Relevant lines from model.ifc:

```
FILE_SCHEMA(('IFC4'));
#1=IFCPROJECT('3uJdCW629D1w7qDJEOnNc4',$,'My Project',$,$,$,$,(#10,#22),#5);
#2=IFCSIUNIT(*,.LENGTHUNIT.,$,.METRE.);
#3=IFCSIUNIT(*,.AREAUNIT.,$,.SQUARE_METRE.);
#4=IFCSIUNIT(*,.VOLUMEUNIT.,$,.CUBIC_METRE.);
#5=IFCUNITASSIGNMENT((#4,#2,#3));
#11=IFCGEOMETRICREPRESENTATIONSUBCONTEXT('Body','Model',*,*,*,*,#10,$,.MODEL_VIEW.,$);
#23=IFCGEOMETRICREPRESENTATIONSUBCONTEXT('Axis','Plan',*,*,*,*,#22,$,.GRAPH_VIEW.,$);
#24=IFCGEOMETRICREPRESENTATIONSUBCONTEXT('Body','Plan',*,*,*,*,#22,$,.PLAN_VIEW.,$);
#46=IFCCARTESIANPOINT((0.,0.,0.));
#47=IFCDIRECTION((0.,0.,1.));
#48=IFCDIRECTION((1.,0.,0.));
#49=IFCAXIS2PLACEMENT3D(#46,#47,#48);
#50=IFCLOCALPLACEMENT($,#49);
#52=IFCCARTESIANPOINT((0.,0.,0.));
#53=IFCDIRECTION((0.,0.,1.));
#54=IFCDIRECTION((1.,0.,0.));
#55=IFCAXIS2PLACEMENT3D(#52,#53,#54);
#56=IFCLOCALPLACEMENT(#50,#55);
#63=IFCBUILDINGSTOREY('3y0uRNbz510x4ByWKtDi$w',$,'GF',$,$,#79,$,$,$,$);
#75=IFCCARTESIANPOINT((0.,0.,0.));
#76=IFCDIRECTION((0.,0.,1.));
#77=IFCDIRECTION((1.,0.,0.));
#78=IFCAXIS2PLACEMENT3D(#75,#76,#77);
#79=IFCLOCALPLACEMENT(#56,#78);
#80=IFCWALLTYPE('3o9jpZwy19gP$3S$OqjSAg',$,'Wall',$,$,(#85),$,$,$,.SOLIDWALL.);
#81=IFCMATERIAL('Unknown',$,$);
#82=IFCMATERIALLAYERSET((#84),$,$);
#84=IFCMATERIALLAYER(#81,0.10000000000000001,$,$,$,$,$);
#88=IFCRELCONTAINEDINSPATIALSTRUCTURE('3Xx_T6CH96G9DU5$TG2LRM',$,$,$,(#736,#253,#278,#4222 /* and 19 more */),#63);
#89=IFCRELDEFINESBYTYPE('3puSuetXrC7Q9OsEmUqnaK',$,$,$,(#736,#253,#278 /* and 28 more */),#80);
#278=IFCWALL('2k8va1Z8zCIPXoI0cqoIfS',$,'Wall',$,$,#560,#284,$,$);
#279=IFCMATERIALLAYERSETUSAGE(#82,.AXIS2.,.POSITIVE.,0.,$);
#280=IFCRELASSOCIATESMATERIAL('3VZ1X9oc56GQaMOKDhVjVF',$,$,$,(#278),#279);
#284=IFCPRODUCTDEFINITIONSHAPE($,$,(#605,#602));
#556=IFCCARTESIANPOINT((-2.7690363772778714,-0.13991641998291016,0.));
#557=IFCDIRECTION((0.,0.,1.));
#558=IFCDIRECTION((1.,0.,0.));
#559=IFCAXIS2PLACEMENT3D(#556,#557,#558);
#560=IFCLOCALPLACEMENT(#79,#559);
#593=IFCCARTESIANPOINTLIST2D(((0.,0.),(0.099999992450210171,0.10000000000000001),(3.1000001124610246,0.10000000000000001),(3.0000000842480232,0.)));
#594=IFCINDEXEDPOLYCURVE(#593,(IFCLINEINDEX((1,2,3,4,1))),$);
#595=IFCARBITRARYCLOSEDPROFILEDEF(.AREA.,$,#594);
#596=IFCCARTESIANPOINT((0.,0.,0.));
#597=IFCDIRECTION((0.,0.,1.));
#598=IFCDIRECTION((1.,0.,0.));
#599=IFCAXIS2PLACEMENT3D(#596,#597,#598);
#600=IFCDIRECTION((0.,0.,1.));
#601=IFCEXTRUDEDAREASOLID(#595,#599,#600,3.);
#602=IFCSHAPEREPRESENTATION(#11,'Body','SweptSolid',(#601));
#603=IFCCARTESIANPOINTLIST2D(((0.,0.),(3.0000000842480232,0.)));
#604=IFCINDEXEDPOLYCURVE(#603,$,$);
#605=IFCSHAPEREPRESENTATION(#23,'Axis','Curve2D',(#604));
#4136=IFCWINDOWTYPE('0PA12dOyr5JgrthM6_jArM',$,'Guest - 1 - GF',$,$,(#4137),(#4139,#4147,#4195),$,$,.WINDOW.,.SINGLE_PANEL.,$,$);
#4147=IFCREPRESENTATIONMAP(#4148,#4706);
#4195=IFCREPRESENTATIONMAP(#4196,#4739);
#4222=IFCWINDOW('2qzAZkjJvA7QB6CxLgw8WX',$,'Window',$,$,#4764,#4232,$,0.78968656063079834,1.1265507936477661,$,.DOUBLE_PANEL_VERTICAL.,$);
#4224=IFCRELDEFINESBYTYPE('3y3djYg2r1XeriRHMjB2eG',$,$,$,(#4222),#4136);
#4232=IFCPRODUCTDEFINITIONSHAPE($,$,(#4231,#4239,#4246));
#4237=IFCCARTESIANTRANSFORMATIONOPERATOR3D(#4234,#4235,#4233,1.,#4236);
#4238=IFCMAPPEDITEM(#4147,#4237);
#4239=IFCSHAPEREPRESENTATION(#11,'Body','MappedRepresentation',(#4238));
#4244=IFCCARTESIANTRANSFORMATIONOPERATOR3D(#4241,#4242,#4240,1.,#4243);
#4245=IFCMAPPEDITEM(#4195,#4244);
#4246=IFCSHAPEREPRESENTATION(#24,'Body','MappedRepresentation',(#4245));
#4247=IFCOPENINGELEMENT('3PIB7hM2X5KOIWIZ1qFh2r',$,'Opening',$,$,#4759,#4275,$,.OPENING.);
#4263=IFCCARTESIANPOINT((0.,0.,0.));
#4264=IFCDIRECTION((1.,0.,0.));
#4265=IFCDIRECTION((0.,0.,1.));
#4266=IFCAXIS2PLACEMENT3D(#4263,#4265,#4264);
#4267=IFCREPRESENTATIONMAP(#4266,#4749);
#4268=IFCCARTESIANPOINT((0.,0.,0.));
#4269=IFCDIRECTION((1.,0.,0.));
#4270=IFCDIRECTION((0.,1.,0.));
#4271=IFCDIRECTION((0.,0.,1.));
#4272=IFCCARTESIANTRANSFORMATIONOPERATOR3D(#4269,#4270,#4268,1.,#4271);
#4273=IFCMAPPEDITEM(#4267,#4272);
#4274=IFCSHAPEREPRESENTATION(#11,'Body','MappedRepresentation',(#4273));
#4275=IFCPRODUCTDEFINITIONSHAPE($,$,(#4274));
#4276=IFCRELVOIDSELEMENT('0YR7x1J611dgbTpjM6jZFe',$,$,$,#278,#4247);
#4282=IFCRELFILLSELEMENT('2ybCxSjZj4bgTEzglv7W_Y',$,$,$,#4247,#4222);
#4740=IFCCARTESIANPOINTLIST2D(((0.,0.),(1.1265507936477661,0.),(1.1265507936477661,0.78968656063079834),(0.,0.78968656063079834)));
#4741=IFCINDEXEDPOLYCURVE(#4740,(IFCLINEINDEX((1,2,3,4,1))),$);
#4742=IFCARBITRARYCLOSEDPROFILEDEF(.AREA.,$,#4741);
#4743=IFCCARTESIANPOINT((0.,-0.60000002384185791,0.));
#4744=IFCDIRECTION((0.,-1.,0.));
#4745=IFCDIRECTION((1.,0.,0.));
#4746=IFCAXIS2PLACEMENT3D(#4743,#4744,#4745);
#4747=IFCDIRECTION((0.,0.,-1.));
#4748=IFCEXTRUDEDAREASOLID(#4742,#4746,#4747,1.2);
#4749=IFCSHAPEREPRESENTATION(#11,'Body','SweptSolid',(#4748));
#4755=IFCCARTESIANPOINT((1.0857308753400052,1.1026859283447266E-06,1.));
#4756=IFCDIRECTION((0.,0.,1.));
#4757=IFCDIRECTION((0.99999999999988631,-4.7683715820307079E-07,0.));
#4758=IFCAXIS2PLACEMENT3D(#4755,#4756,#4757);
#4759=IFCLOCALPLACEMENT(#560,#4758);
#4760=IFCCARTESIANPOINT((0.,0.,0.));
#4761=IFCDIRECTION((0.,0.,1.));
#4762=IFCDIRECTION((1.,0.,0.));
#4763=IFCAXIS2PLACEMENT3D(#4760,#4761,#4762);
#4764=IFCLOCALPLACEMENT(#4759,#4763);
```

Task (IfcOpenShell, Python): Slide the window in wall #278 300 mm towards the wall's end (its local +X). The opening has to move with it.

```python
import ifcopenshell
import ifcopenshell.api.geometry
import ifcopenshell.util.placement

model = ifcopenshell.open("model.ifc")

window = model.by_guid("2qzAZkjJvA7QB6CxLgw8WX")
opening = window.FillsVoids[0].RelatingOpeningElement
wall = opening.VoidsElements[0].RelatingBuildingElement

wall_matrix = ifcopenshell.util.placement.get_local_placement(wall.ObjectPlacement)
shift = wall_matrix[:3, 0] * 0.3
before = ifcopenshell.util.placement.get_local_placement(window.ObjectPlacement)[:3, 3].copy()

# The window is placed relative to its opening, so it follows when the opening moves.
matrix = ifcopenshell.util.placement.get_local_placement(opening.ObjectPlacement)
matrix[:3, 3] += shift
ifcopenshell.api.geometry.edit_object_placement(
    model, product=opening, matrix=matrix, is_si=False, should_transform_children=True
)

after = ifcopenshell.util.placement.get_local_placement(window.ObjectPlacement)[:3, 3]
print("window moved by", (after - before).round(3) + 0.0)

model.write("model_edited.ifc")
```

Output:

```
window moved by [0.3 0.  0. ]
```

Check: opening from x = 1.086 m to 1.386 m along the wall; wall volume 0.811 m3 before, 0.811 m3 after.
